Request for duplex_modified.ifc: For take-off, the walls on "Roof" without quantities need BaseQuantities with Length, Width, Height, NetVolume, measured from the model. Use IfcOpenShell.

First a look at what the model holds.

```python
import ifcopenshell
import ifcopenshell.util.element
import ifcopenshell.util.unit

model = ifcopenshell.open("duplex_modified.ifc")
print(model.schema)
for unit_type in ("LENGTHUNIT", "AREAUNIT", "VOLUMEUNIT"):
    print(unit_type, ifcopenshell.util.unit.calculate_unit_scale(model, unit_type))
storey = next(s for s in model.by_type("IfcBuildingStorey") if s.Name == "Roof")
walls = [e for e in ifcopenshell.util.element.get_decomposition(storey) if e.is_a("IfcWall")]
for e in sorted(walls, key=lambda e: e.id()):
    print(e.id(), e.is_a(), e.Name, list(ifcopenshell.util.element.get_psets(e, qtos_only=True)), sep=" | ")
```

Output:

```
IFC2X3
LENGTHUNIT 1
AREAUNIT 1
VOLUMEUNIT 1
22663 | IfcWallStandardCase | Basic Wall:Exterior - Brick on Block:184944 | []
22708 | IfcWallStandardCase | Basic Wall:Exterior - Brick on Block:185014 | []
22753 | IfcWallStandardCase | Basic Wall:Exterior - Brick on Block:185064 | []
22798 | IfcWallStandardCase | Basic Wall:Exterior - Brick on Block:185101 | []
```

```python
import ifcopenshell
import ifcopenshell.api.pset
import ifcopenshell.geom
import ifcopenshell.util.element
import ifcopenshell.util.shape
import ifcopenshell.util.unit

model = ifcopenshell.open("duplex_modified.ifc")
unit_scale = ifcopenshell.util.unit.calculate_unit_scale(model)
volume_scale = ifcopenshell.util.unit.calculate_unit_scale(model, "VOLUMEUNIT")
settings = ifcopenshell.geom.settings()

storey = next(s for s in model.by_type("IfcBuildingStorey") if s.Name == "Roof")
walls = [e for e in ifcopenshell.util.element.get_decomposition(storey) if e.is_a("IfcWall")]

for e in sorted(walls, key=lambda e: e.id()):
    if ifcopenshell.util.element.get_psets(e, qtos_only=True, should_inherit=False):
        continue
    # Geometry comes back in metres, in the element's own axes.
    shape = ifcopenshell.geom.create_shape(settings, e)
    values = {
        "Length": ifcopenshell.util.shape.get_x(shape.geometry) / unit_scale,
        "Width": ifcopenshell.util.shape.get_y(shape.geometry) / unit_scale,
        "Height": ifcopenshell.util.shape.get_z(shape.geometry) / unit_scale,
        "NetVolume": ifcopenshell.util.shape.get_volume(shape.geometry) / volume_scale,
    }
    qto = ifcopenshell.api.pset.add_qto(model, product=e, name="BaseQuantities")
    ifcopenshell.api.pset.edit_qto(model, qto=qto, properties=values)
    print(e.id(), {k: round(v, 3) for k, v in values.items()})

model.write("duplex_modified_rev.ifc")
```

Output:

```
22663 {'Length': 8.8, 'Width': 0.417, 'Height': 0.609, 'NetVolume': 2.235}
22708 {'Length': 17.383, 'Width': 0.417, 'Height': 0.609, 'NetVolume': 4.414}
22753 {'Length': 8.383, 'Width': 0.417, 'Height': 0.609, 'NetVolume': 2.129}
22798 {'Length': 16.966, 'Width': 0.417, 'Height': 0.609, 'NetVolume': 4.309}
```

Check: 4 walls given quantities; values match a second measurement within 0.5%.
